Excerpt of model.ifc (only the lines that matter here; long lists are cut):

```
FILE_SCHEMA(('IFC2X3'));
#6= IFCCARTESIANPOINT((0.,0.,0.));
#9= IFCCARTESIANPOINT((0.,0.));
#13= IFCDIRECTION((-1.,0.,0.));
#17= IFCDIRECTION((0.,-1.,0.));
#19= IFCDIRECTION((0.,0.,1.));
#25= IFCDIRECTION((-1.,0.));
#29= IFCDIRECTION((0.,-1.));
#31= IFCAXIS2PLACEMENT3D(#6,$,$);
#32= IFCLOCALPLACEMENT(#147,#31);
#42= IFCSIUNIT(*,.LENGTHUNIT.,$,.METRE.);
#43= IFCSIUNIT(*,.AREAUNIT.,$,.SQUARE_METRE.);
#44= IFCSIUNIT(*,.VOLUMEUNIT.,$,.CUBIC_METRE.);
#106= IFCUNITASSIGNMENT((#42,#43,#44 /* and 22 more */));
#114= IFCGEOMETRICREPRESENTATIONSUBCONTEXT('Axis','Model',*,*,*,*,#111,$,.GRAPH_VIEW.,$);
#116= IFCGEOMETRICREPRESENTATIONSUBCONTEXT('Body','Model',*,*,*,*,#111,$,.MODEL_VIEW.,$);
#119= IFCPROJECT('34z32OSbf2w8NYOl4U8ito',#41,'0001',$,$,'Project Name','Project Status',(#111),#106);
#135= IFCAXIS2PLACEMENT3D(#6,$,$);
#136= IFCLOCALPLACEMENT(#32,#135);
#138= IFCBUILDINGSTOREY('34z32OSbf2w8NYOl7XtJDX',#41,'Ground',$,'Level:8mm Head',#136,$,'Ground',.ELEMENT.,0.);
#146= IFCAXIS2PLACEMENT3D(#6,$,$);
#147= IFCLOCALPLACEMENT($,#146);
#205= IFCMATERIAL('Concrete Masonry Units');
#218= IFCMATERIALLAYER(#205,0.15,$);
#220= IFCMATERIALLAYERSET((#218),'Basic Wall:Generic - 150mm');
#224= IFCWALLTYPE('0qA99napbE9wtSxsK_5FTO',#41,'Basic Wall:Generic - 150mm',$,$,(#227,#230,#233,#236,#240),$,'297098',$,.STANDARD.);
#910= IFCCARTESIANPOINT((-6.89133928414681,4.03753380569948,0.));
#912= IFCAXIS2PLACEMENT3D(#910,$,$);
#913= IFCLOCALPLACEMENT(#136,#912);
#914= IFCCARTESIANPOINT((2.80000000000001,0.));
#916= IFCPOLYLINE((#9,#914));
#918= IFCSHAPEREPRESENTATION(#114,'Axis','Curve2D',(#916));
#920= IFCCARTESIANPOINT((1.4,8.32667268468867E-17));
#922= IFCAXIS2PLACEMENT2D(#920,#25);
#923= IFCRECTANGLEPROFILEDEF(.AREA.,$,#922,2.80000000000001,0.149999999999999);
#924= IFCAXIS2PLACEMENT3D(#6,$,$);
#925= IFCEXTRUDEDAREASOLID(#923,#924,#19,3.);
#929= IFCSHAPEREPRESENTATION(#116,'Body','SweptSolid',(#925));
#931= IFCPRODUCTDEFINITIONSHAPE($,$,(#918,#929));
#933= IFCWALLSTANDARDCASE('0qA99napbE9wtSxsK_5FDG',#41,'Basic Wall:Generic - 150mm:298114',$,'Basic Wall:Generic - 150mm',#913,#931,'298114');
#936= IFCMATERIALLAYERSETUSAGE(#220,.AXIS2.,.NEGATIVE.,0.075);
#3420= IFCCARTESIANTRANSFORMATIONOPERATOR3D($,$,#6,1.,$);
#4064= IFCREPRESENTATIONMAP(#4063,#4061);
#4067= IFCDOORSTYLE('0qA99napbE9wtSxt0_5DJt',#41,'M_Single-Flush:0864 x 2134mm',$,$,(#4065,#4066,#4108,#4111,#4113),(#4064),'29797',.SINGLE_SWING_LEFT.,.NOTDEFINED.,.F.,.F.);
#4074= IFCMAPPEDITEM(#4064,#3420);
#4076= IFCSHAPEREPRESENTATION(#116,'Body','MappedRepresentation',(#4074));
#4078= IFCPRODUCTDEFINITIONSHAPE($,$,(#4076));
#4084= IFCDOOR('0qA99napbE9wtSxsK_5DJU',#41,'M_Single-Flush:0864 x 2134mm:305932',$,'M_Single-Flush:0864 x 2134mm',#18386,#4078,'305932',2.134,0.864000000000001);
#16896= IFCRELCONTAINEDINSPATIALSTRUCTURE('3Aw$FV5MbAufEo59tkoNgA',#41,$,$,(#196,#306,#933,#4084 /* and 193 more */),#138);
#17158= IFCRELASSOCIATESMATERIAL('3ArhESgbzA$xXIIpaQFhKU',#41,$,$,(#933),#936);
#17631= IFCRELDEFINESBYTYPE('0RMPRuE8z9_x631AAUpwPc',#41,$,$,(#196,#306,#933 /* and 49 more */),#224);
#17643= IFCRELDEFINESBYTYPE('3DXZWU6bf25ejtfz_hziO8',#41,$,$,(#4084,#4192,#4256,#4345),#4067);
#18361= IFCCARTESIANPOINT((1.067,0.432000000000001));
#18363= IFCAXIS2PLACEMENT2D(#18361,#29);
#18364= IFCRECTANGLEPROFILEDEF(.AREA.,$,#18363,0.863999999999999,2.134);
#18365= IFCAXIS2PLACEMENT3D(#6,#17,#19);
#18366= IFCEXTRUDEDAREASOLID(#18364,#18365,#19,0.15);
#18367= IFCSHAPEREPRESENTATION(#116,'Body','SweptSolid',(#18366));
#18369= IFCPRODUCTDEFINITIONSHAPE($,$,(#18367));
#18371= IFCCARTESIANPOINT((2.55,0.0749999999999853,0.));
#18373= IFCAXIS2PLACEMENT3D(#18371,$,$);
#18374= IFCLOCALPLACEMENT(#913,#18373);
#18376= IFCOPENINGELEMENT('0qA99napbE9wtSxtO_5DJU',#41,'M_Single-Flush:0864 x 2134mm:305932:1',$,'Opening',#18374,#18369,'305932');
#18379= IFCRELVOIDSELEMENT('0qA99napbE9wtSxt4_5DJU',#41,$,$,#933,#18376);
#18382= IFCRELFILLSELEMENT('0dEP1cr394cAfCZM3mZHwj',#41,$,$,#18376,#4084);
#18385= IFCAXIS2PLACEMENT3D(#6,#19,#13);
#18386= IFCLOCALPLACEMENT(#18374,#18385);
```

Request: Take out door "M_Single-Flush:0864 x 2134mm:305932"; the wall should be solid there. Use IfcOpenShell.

```python
import ifcopenshell
import ifcopenshell.api.feature
import ifcopenshell.api.root
import ifcopenshell.geom
import ifcopenshell.util.shape

model = ifcopenshell.open("model.ifc")
settings = ifcopenshell.geom.settings()


def volume(element):
    """Net volume in cubic metres, openings subtracted."""
    shape = ifcopenshell.geom.create_shape(settings, element)
    return ifcopenshell.util.shape.get_volume(shape.geometry)


door = model.by_guid("0qA99napbE9wtSxsK_5DJU")
opening = door.FillsVoids[0].RelatingOpeningElement
wall = opening.VoidsElements[0].RelatingBuildingElement
before = volume(wall)

ifcopenshell.api.root.remove_product(model, product=door)
ifcopenshell.api.feature.remove_feature(model, feature=opening)

after = volume(wall)

print(f"wall volume {before:.3f} -> {after:.3f} m3")

model.write("model_rev.ifc")
```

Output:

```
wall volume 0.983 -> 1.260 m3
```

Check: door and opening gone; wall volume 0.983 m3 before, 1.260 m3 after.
